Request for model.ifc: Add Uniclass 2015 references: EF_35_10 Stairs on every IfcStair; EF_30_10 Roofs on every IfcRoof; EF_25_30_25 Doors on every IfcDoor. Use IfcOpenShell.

First a look at what the model holds.

```python
import ifcopenshell

model = ifcopenshell.open("model.ifc")
print(model.schema)
print("classifications:", [c.Name for c in model.by_type("IfcClassification")])
for ifc_class in ("IfcDoor", "IfcRoof", "IfcStair", "IfcWall", "IfcWindow"):
    print(ifc_class, len(model.by_type(ifc_class)))
```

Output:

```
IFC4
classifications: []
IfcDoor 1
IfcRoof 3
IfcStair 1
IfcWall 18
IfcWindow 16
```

```python
import ifcopenshell
import ifcopenshell.api.classification

model = ifcopenshell.open("model.ifc")

system = ifcopenshell.api.classification.add_classification(model, classification="Uniclass 2015")

codes = {
    "IfcStair": ("EF_35_10", "Stairs"),
    "IfcRoof": ("EF_30_10", "Roofs"),
    "IfcDoor": ("EF_25_30_25", "Doors"),
}
for ifc_class, (code, name) in codes.items():
    products = model.by_type(ifc_class)
    ifcopenshell.api.classification.add_reference(
        model, products=products, classification=system, identification=code, name=name
    )
    print(code, len(products))

model.write("model-out.ifc")
```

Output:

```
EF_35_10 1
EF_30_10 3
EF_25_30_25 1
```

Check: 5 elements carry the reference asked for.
